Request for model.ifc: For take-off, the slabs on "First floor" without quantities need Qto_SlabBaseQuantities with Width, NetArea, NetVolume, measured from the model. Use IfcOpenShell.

First a look at what the model holds.

```python
import ifcopenshell
import ifcopenshell.util.element
import ifcopenshell.util.unit

model = ifcopenshell.open("model.ifc")
print(model.schema)
for unit_type in ("LENGTHUNIT", "AREAUNIT", "VOLUMEUNIT"):
    print(unit_type, ifcopenshell.util.unit.calculate_unit_scale(model, unit_type))
storey = next(s for s in model.by_type("IfcBuildingStorey") if s.Name == "First floor")
slabs = [e for e in ifcopenshell.util.element.get_decomposition(storey) if e.is_a("IfcSlab")]
for e in sorted(slabs, key=lambda e: e.id()):
    print(e.id(), e.is_a(), e.Name, list(ifcopenshell.util.element.get_psets(e, qtos_only=True)), sep=" | ")
```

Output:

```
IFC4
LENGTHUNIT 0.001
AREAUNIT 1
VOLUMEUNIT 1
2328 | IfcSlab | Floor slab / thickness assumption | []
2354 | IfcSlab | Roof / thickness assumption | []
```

```python
import ifcopenshell
import ifcopenshell.api.pset
import ifcopenshell.geom
import ifcopenshell.util.element
import ifcopenshell.util.shape
import ifcopenshell.util.unit

model = ifcopenshell.open("model.ifc")
unit_scale = ifcopenshell.util.unit.calculate_unit_scale(model)
area_scale = ifcopenshell.util.unit.calculate_unit_scale(model, "AREAUNIT")
volume_scale = ifcopenshell.util.unit.calculate_unit_scale(model, "VOLUMEUNIT")
settings = ifcopenshell.geom.settings()

storey = next(s for s in model.by_type("IfcBuildingStorey") if s.Name == "First floor")
slabs = [e for e in ifcopenshell.util.element.get_decomposition(storey) if e.is_a("IfcSlab")]

for e in sorted(slabs, key=lambda e: e.id()):
    if ifcopenshell.util.element.get_psets(e, qtos_only=True, should_inherit=False):
        continue
    # Geometry comes back in metres, in the element's own axes.
    shape = ifcopenshell.geom.create_shape(settings, e)
    values = {
        "Width": ifcopenshell.util.shape.get_z(shape.geometry) / unit_scale,
        "NetArea": ifcopenshell.util.shape.get_footprint_area(shape.geometry) / area_scale,
        "NetVolume": ifcopenshell.util.shape.get_volume(shape.geometry) / volume_scale,
    }
    qto = ifcopenshell.api.pset.add_qto(model, product=e, name="Qto_SlabBaseQuantities")
    ifcopenshell.api.pset.edit_qto(model, qto=qto, properties=values)
    print(e.id(), {k: round(v, 3) for k, v in values.items()})

model.write("model_v2.ifc")
```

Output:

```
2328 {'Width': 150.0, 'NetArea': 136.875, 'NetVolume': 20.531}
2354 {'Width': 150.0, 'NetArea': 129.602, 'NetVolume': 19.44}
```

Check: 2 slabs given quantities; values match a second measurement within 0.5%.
